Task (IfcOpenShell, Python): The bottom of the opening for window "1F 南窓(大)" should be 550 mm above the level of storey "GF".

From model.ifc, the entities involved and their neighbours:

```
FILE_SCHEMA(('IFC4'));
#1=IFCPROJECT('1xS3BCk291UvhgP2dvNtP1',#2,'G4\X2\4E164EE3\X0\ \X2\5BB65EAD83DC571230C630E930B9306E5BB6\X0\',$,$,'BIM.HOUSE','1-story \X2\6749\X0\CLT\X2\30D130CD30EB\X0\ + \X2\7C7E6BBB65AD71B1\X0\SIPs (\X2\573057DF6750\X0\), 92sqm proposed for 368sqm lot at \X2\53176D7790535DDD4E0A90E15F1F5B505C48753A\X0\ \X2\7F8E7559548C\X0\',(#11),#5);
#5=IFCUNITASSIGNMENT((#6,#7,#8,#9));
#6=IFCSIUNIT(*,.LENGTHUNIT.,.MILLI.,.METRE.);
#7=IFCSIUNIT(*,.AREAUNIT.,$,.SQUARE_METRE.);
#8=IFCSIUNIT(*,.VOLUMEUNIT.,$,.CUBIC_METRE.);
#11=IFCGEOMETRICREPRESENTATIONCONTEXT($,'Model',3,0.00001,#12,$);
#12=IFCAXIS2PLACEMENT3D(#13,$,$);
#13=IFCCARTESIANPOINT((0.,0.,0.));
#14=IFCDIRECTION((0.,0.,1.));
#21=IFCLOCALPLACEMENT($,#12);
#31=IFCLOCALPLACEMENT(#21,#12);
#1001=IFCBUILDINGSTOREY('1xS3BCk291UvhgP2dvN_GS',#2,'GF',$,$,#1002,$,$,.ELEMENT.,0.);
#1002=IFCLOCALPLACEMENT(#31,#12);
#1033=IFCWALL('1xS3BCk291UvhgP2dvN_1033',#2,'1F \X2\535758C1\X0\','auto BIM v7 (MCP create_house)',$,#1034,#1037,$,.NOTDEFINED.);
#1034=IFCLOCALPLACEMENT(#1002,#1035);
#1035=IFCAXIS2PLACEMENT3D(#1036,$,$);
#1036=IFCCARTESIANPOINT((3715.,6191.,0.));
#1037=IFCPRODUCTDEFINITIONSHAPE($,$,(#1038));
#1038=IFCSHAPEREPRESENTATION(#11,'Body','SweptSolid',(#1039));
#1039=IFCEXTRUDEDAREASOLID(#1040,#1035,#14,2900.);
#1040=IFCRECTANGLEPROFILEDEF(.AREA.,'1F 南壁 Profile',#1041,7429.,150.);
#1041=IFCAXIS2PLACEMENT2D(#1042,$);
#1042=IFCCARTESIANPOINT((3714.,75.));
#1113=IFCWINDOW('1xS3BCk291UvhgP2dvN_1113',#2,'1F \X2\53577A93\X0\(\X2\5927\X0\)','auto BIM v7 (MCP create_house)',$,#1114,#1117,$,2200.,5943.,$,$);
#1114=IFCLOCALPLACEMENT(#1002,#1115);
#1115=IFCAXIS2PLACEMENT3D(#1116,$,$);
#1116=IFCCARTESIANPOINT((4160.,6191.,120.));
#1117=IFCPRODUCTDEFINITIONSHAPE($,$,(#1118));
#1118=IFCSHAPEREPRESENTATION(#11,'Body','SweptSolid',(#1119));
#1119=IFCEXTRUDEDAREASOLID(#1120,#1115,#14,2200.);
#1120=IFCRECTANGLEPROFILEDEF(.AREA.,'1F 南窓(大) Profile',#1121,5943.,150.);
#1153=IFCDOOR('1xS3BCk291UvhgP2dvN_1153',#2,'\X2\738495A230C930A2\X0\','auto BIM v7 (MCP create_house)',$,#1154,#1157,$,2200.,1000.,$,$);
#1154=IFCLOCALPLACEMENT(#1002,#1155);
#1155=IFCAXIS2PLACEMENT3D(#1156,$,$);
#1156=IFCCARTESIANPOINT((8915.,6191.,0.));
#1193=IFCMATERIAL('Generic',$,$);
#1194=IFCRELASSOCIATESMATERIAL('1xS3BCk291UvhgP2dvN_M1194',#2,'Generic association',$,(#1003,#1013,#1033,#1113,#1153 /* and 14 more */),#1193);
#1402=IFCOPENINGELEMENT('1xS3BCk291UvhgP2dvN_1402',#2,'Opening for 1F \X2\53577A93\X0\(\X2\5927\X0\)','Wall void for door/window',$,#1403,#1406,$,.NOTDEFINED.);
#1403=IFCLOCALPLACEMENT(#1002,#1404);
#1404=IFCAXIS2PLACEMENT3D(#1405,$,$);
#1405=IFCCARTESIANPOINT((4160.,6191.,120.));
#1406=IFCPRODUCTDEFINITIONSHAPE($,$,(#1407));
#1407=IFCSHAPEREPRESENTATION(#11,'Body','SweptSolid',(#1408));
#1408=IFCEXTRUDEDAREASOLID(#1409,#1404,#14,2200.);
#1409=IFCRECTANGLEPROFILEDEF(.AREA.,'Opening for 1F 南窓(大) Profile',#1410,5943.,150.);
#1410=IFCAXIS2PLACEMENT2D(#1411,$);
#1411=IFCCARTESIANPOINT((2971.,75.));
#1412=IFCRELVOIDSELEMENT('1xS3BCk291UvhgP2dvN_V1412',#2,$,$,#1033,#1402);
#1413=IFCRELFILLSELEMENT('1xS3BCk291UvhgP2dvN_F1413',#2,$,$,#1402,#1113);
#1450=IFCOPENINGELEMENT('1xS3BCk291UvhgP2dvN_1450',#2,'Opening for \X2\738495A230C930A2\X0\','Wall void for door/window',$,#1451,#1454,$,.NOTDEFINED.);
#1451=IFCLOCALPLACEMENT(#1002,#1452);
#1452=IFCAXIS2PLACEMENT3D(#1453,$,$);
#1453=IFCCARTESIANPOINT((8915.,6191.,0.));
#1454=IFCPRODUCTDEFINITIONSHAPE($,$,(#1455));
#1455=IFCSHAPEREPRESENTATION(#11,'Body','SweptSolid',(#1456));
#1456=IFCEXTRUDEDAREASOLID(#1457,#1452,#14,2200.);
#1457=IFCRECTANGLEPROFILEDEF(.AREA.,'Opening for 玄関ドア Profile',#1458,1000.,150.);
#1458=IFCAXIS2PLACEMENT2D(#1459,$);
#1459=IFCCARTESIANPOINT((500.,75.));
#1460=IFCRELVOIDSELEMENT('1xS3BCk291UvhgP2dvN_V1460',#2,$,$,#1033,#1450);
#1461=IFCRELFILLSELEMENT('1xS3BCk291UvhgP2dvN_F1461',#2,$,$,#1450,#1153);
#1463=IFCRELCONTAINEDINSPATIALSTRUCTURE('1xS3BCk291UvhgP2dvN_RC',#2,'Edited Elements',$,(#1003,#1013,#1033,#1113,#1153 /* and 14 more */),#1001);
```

```python
import numpy as np
import ifcopenshell
import ifcopenshell.api.geometry
import ifcopenshell.geom
import ifcopenshell.util.element
import ifcopenshell.util.placement
import ifcopenshell.util.shape
import ifcopenshell.util.unit

model = ifcopenshell.open("model.ifc")
unit_scale = ifcopenshell.util.unit.calculate_unit_scale(model)

window = model.by_guid("1xS3BCk291UvhgP2dvN_1113")
opening = window.FillsVoids[0].RelatingOpeningElement
storey = ifcopenshell.util.element.get_container(window, ifc_class="IfcBuildingStorey")
level = ifcopenshell.util.placement.get_local_placement(storey.ObjectPlacement)[2, 3]

# The opening's origin need not be at the sill, so measure its lowest point.
shape = ifcopenshell.geom.create_shape(ifcopenshell.geom.settings(), opening)
bottom = ifcopenshell.util.shape.get_shape_bottom_elevation(shape, shape.geometry) / unit_scale
dz = level + 0.55 / unit_scale - bottom

shift = np.array([0.0, 0.0, dz])
# The window is not placed relative to its opening, so move both.
for product in (opening, window):
    matrix = ifcopenshell.util.placement.get_local_placement(product.ObjectPlacement)
    matrix[:3, 3] += shift
    ifcopenshell.api.geometry.edit_object_placement(model, product=product, matrix=matrix, is_si=False)

print(f"moved by {dz * unit_scale:+.3f} m")

model.write("model_v2.ifc")
```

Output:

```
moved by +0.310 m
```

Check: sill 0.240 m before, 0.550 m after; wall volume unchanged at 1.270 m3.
